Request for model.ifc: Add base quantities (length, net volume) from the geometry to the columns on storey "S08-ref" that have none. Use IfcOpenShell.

First a look at what the model holds.

```python
import ifcopenshell
import ifcopenshell.util.element
import ifcopenshell.util.unit

model = ifcopenshell.open("model.ifc")
print(model.schema)
for unit_type in ("LENGTHUNIT", "AREAUNIT", "VOLUMEUNIT"):
    print(unit_type, ifcopenshell.util.unit.calculate_unit_scale(model, unit_type))
storey = next(s for s in model.by_type("IfcBuildingStorey") if s.Name == "S08-ref")
columns = [e for e in ifcopenshell.util.element.get_decomposition(storey) if e.is_a("IfcColumn")]
for e in sorted(columns, key=lambda e: e.id()):
    print(e.id(), e.is_a(), e.Name, list(ifcopenshell.util.element.get_psets(e, qtos_only=True)), sep=" | ")
```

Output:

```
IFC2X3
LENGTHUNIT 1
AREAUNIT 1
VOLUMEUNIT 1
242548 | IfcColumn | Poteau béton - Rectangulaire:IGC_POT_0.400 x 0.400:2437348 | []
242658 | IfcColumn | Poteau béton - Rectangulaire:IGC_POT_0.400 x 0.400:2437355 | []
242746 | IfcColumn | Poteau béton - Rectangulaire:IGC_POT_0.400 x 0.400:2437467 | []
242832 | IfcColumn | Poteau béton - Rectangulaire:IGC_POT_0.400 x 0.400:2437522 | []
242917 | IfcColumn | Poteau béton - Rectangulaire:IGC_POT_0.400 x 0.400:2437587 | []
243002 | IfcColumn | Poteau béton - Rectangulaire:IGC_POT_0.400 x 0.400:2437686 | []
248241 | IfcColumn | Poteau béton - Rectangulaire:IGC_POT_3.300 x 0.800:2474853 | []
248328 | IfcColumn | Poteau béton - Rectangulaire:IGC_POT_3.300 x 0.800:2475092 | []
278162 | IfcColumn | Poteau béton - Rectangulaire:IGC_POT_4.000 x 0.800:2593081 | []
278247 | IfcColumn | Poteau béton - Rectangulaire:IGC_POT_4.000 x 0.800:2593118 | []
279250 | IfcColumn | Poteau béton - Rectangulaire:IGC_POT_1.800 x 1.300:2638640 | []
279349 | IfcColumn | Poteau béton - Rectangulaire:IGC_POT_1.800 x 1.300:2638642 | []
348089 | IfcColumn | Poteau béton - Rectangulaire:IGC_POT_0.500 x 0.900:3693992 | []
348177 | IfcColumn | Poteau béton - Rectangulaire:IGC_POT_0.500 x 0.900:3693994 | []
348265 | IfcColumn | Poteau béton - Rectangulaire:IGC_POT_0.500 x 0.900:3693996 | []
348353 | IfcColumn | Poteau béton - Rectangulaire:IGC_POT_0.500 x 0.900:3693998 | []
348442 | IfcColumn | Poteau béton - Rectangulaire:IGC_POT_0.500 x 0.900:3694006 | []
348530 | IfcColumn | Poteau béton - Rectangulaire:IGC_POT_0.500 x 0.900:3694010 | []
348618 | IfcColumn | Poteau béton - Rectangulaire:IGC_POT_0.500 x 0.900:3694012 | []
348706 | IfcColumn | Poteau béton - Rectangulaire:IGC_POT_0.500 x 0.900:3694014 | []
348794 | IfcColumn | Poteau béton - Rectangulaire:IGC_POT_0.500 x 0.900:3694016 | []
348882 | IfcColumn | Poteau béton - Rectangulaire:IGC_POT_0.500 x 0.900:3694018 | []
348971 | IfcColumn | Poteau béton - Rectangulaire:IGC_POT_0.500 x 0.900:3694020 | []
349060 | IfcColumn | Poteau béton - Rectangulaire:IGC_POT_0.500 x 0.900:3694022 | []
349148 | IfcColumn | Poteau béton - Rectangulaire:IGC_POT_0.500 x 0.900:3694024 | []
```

```python
import ifcopenshell
import ifcopenshell.api.pset
import ifcopenshell.geom
import ifcopenshell.util.element
import ifcopenshell.util.shape
import ifcopenshell.util.unit

model = ifcopenshell.open("model.ifc")
unit_scale = ifcopenshell.util.unit.calculate_unit_scale(model)
volume_scale = ifcopenshell.util.unit.calculate_unit_scale(model, "VOLUMEUNIT")
settings = ifcopenshell.geom.settings()

storey = next(s for s in model.by_type("IfcBuildingStorey") if s.Name == "S08-ref")
columns = [e for e in ifcopenshell.util.element.get_decomposition(storey) if e.is_a("IfcColumn")]

for e in sorted(columns, key=lambda e: e.id()):
    if ifcopenshell.util.element.get_psets(e, qtos_only=True, should_inherit=False):
        continue
    # Geometry comes back in metres, in the element's own axes.
    shape = ifcopenshell.geom.create_shape(settings, e)
    values = {
        "Length": ifcopenshell.util.shape.get_z(shape.geometry) / unit_scale,
        "NetVolume": ifcopenshell.util.shape.get_volume(shape.geometry) / volume_scale,
    }
    qto = ifcopenshell.api.pset.add_qto(model, product=e, name="BaseQuantities")
    ifcopenshell.api.pset.edit_qto(model, qto=qto, properties=values)
    print(e.id(), {k: round(v, 3) for k, v in values.items()})

model.write("model_rev.ifc")
```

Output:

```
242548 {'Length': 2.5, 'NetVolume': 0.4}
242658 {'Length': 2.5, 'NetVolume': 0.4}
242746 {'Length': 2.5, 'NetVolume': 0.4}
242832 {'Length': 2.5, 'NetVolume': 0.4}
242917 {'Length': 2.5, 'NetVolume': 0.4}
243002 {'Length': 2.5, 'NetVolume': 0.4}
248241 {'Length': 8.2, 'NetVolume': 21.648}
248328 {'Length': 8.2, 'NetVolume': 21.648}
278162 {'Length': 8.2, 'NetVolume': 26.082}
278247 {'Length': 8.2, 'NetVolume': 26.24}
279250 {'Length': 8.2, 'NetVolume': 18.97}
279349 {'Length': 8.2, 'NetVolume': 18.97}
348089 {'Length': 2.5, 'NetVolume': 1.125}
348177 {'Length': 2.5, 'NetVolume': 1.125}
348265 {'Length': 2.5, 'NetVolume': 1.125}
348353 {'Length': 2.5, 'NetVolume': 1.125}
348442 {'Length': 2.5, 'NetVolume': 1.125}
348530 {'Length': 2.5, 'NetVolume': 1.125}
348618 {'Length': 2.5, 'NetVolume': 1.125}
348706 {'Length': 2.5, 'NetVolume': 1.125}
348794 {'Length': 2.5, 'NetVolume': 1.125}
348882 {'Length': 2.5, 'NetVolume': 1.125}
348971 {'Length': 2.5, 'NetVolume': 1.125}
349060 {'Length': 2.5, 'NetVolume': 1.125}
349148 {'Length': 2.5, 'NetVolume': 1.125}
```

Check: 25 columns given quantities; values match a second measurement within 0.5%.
